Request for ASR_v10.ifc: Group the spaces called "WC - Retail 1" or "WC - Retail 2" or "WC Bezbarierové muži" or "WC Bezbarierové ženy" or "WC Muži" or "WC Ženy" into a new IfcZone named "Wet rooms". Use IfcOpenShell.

First a look at what the model holds.

```python
import ifcopenshell

model = ifcopenshell.open("ASR_v10.ifc")
print(model.schema)
seen = {}
for space in model.by_type("IfcSpace"):
    seen[space.LongName] = seen.get(space.LongName, 0) + 1
for name, count in sorted(seen.items(), key=str):
    print(count, "x", name)
print("zones:", [z.Name for z in model.by_type("IfcZone")][:20])
```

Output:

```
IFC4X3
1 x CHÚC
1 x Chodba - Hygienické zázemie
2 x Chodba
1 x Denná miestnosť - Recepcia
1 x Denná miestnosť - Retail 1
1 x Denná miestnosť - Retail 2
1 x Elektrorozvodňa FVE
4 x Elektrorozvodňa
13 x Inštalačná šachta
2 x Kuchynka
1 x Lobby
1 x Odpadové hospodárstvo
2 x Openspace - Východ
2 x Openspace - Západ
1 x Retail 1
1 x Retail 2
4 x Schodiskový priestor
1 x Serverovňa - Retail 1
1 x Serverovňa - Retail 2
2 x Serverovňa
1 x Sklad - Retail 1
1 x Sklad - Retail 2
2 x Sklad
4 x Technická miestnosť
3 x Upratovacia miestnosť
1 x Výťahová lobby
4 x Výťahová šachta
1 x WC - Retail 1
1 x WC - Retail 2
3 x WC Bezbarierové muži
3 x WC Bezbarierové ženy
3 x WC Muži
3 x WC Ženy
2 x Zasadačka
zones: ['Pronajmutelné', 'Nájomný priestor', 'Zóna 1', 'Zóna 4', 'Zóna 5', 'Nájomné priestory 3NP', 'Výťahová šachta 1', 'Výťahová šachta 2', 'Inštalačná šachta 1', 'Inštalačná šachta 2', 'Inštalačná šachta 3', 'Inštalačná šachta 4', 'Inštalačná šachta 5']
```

```python
import ifcopenshell
import ifcopenshell.api.group
import ifcopenshell.api.root

model = ifcopenshell.open("ASR_v10.ifc")

names = {"WC - Retail 1", "WC - Retail 2", "WC Bezbarierové muži", "WC Bezbarierové ženy", "WC Muži", "WC Ženy"}
spaces = [s for s in model.by_type("IfcSpace") if s.LongName in names]

zone = ifcopenshell.api.root.create_entity(model, ifc_class="IfcZone", name="Wet rooms")
ifcopenshell.api.group.assign_group(model, products=spaces, group=zone)
print(len(spaces), "spaces in", zone.Name)

model.write("ASR_v10_edited.ifc")
```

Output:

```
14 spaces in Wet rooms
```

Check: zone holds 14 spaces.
